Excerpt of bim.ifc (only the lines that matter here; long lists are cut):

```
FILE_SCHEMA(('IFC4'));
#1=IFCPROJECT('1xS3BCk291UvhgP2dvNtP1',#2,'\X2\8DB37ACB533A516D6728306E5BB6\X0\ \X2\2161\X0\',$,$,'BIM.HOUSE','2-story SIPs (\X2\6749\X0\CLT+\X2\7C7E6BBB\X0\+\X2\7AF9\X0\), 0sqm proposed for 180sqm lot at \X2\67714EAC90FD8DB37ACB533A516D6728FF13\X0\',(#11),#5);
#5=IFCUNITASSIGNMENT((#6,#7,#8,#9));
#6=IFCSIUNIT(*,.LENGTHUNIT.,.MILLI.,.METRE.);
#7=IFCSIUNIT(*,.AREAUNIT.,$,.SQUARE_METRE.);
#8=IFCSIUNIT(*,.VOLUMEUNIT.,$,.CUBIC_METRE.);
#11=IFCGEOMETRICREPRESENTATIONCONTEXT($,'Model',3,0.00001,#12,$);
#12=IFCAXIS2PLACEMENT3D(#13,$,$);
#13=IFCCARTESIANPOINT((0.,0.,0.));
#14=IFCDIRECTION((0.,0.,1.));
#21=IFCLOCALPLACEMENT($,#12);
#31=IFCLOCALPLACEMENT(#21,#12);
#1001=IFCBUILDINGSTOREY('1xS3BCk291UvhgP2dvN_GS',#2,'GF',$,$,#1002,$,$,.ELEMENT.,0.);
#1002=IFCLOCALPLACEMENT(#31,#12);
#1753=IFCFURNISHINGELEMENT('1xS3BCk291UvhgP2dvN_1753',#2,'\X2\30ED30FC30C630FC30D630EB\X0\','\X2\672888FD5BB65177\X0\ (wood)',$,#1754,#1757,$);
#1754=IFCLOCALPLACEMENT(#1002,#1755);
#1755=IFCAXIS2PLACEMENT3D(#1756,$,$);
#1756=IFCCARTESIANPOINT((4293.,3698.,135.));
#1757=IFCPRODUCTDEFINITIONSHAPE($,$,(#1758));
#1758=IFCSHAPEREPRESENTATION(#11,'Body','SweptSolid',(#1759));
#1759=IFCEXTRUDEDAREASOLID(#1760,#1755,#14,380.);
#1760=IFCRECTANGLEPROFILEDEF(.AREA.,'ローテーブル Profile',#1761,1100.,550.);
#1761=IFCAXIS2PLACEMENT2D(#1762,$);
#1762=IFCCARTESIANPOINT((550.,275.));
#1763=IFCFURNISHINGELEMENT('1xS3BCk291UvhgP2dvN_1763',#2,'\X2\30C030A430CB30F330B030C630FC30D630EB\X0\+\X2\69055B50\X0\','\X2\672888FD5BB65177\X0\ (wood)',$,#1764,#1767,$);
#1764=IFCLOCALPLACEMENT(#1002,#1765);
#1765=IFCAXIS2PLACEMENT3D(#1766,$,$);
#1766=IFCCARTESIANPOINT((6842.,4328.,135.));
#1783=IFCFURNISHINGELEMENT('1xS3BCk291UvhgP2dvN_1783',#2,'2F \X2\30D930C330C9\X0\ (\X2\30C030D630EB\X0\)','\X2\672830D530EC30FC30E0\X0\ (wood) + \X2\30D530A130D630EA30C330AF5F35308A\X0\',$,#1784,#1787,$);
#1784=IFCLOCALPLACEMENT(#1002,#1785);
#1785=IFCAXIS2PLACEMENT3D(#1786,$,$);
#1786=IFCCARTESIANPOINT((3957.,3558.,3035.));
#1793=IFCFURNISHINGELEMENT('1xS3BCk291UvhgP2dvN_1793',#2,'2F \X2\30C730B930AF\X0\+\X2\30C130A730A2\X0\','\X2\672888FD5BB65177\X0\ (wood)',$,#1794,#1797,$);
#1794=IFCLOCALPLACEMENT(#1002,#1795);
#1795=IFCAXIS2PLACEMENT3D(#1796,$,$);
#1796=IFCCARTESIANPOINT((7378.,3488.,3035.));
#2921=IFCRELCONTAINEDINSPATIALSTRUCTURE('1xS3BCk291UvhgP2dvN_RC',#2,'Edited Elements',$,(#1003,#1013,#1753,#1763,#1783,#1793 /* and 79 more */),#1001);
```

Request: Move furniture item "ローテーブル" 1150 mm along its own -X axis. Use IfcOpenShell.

```python
import ifcopenshell
import ifcopenshell.api.geometry
import ifcopenshell.util.placement
import ifcopenshell.util.unit

model = ifcopenshell.open("bim.ifc")
unit_scale = ifcopenshell.util.unit.calculate_unit_scale(model)

item = model.by_id(1753)
matrix = ifcopenshell.util.placement.get_local_placement(item.ObjectPlacement)
matrix[:3, 3] -= matrix[:3, 0] * 1.15 / unit_scale
ifcopenshell.api.geometry.edit_object_placement(model, product=item, matrix=matrix, is_si=False)

print(ifcopenshell.util.placement.get_local_placement(item.ObjectPlacement).round(3) + 0.0)

model.write("bim_updated.ifc")
```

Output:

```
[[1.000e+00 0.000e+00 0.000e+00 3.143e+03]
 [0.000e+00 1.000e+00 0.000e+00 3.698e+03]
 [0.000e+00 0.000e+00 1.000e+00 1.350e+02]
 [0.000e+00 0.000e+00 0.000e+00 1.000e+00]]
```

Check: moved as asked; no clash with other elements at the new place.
